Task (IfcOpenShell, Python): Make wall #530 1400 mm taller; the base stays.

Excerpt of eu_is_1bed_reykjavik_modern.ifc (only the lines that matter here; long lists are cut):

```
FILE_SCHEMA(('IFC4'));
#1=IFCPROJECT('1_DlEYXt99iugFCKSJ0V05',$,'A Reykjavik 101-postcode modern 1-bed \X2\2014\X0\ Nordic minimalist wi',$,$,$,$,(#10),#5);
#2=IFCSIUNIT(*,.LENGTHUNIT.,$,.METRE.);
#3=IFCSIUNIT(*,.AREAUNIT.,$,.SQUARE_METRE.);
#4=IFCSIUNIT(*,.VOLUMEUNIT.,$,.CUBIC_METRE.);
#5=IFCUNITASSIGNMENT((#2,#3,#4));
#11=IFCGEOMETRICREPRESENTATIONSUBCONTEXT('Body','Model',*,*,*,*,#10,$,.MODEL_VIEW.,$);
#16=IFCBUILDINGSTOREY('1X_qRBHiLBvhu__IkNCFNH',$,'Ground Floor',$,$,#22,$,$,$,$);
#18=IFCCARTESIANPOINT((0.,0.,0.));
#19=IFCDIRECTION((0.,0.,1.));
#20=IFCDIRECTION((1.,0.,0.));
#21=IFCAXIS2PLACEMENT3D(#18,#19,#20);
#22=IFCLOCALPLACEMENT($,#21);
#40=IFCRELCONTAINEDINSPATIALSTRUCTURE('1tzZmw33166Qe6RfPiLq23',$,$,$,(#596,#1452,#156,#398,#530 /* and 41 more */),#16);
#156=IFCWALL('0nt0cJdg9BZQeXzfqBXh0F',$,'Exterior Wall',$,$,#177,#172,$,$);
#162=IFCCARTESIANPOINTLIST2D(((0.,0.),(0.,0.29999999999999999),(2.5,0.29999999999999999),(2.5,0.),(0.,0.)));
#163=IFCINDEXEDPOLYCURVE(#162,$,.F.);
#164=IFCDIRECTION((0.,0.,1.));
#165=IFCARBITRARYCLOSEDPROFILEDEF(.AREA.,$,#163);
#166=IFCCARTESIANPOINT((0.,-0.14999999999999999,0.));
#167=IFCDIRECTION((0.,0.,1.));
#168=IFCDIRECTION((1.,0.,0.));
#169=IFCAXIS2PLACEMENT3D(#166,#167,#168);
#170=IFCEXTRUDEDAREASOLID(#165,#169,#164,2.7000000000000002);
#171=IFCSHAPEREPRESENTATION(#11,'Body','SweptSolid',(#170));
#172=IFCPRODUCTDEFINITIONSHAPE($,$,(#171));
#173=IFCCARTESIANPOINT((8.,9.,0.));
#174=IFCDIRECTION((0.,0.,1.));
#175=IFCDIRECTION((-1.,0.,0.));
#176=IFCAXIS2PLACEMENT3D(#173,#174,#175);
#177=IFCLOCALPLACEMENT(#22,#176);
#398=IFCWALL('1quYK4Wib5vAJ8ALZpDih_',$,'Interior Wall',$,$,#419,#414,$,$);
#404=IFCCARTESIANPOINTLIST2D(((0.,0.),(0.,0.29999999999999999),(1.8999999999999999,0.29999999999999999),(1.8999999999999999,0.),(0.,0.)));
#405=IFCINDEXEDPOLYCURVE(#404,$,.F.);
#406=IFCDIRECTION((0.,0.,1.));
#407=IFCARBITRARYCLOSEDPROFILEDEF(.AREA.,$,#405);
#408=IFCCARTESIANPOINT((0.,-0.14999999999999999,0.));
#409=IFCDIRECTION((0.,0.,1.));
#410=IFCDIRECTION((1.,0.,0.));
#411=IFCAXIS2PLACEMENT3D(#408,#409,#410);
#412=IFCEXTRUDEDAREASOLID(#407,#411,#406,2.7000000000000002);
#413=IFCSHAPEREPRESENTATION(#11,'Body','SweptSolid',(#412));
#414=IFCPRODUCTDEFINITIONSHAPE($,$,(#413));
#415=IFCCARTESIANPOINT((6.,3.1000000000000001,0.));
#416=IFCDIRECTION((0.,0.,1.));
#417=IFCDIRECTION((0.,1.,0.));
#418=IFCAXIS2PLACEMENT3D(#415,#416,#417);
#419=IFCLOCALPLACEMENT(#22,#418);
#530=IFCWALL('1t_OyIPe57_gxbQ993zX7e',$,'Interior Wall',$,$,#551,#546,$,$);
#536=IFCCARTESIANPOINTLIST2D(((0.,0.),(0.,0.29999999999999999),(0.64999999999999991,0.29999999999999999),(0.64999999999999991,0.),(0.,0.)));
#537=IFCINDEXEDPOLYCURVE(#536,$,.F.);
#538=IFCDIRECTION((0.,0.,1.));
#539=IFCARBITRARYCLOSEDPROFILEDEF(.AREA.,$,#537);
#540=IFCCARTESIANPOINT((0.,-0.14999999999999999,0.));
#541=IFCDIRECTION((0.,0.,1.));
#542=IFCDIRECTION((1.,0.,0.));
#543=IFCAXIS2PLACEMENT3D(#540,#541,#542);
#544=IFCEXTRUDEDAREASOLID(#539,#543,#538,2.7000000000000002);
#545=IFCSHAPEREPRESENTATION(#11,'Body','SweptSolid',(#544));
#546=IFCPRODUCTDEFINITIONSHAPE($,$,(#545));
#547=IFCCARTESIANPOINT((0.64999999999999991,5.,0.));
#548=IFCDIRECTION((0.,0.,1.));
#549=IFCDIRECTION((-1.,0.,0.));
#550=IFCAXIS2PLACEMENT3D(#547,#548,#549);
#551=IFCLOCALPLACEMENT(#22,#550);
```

```python
import ifcopenshell
import ifcopenshell.geom
import ifcopenshell.util.representation
import ifcopenshell.util.shape
import ifcopenshell.util.unit

model = ifcopenshell.open("eu_is_1bed_reykjavik_modern.ifc")
unit_scale = ifcopenshell.util.unit.calculate_unit_scale(model)
settings = ifcopenshell.geom.settings()


def volume(element):
    """Net volume in cubic metres, openings subtracted."""
    shape = ifcopenshell.geom.create_shape(settings, element)
    return ifcopenshell.util.shape.get_volume(shape.geometry)


wall = model.by_id(530)
before = volume(wall)

body = ifcopenshell.util.representation.get_representation(wall, "Model", "Body")
solid = body.Items[0]
old_height = solid.Depth
solid.Depth += 1.4 / unit_scale
after = volume(wall)

print(f"height {old_height:g} -> {solid.Depth:g}, volume {before:.3f} -> {after:.3f} m3")

model.write("eu_is_1bed_reykjavik_modern_v2.ifc")
```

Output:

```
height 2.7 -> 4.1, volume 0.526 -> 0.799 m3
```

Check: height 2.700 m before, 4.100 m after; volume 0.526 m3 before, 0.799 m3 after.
